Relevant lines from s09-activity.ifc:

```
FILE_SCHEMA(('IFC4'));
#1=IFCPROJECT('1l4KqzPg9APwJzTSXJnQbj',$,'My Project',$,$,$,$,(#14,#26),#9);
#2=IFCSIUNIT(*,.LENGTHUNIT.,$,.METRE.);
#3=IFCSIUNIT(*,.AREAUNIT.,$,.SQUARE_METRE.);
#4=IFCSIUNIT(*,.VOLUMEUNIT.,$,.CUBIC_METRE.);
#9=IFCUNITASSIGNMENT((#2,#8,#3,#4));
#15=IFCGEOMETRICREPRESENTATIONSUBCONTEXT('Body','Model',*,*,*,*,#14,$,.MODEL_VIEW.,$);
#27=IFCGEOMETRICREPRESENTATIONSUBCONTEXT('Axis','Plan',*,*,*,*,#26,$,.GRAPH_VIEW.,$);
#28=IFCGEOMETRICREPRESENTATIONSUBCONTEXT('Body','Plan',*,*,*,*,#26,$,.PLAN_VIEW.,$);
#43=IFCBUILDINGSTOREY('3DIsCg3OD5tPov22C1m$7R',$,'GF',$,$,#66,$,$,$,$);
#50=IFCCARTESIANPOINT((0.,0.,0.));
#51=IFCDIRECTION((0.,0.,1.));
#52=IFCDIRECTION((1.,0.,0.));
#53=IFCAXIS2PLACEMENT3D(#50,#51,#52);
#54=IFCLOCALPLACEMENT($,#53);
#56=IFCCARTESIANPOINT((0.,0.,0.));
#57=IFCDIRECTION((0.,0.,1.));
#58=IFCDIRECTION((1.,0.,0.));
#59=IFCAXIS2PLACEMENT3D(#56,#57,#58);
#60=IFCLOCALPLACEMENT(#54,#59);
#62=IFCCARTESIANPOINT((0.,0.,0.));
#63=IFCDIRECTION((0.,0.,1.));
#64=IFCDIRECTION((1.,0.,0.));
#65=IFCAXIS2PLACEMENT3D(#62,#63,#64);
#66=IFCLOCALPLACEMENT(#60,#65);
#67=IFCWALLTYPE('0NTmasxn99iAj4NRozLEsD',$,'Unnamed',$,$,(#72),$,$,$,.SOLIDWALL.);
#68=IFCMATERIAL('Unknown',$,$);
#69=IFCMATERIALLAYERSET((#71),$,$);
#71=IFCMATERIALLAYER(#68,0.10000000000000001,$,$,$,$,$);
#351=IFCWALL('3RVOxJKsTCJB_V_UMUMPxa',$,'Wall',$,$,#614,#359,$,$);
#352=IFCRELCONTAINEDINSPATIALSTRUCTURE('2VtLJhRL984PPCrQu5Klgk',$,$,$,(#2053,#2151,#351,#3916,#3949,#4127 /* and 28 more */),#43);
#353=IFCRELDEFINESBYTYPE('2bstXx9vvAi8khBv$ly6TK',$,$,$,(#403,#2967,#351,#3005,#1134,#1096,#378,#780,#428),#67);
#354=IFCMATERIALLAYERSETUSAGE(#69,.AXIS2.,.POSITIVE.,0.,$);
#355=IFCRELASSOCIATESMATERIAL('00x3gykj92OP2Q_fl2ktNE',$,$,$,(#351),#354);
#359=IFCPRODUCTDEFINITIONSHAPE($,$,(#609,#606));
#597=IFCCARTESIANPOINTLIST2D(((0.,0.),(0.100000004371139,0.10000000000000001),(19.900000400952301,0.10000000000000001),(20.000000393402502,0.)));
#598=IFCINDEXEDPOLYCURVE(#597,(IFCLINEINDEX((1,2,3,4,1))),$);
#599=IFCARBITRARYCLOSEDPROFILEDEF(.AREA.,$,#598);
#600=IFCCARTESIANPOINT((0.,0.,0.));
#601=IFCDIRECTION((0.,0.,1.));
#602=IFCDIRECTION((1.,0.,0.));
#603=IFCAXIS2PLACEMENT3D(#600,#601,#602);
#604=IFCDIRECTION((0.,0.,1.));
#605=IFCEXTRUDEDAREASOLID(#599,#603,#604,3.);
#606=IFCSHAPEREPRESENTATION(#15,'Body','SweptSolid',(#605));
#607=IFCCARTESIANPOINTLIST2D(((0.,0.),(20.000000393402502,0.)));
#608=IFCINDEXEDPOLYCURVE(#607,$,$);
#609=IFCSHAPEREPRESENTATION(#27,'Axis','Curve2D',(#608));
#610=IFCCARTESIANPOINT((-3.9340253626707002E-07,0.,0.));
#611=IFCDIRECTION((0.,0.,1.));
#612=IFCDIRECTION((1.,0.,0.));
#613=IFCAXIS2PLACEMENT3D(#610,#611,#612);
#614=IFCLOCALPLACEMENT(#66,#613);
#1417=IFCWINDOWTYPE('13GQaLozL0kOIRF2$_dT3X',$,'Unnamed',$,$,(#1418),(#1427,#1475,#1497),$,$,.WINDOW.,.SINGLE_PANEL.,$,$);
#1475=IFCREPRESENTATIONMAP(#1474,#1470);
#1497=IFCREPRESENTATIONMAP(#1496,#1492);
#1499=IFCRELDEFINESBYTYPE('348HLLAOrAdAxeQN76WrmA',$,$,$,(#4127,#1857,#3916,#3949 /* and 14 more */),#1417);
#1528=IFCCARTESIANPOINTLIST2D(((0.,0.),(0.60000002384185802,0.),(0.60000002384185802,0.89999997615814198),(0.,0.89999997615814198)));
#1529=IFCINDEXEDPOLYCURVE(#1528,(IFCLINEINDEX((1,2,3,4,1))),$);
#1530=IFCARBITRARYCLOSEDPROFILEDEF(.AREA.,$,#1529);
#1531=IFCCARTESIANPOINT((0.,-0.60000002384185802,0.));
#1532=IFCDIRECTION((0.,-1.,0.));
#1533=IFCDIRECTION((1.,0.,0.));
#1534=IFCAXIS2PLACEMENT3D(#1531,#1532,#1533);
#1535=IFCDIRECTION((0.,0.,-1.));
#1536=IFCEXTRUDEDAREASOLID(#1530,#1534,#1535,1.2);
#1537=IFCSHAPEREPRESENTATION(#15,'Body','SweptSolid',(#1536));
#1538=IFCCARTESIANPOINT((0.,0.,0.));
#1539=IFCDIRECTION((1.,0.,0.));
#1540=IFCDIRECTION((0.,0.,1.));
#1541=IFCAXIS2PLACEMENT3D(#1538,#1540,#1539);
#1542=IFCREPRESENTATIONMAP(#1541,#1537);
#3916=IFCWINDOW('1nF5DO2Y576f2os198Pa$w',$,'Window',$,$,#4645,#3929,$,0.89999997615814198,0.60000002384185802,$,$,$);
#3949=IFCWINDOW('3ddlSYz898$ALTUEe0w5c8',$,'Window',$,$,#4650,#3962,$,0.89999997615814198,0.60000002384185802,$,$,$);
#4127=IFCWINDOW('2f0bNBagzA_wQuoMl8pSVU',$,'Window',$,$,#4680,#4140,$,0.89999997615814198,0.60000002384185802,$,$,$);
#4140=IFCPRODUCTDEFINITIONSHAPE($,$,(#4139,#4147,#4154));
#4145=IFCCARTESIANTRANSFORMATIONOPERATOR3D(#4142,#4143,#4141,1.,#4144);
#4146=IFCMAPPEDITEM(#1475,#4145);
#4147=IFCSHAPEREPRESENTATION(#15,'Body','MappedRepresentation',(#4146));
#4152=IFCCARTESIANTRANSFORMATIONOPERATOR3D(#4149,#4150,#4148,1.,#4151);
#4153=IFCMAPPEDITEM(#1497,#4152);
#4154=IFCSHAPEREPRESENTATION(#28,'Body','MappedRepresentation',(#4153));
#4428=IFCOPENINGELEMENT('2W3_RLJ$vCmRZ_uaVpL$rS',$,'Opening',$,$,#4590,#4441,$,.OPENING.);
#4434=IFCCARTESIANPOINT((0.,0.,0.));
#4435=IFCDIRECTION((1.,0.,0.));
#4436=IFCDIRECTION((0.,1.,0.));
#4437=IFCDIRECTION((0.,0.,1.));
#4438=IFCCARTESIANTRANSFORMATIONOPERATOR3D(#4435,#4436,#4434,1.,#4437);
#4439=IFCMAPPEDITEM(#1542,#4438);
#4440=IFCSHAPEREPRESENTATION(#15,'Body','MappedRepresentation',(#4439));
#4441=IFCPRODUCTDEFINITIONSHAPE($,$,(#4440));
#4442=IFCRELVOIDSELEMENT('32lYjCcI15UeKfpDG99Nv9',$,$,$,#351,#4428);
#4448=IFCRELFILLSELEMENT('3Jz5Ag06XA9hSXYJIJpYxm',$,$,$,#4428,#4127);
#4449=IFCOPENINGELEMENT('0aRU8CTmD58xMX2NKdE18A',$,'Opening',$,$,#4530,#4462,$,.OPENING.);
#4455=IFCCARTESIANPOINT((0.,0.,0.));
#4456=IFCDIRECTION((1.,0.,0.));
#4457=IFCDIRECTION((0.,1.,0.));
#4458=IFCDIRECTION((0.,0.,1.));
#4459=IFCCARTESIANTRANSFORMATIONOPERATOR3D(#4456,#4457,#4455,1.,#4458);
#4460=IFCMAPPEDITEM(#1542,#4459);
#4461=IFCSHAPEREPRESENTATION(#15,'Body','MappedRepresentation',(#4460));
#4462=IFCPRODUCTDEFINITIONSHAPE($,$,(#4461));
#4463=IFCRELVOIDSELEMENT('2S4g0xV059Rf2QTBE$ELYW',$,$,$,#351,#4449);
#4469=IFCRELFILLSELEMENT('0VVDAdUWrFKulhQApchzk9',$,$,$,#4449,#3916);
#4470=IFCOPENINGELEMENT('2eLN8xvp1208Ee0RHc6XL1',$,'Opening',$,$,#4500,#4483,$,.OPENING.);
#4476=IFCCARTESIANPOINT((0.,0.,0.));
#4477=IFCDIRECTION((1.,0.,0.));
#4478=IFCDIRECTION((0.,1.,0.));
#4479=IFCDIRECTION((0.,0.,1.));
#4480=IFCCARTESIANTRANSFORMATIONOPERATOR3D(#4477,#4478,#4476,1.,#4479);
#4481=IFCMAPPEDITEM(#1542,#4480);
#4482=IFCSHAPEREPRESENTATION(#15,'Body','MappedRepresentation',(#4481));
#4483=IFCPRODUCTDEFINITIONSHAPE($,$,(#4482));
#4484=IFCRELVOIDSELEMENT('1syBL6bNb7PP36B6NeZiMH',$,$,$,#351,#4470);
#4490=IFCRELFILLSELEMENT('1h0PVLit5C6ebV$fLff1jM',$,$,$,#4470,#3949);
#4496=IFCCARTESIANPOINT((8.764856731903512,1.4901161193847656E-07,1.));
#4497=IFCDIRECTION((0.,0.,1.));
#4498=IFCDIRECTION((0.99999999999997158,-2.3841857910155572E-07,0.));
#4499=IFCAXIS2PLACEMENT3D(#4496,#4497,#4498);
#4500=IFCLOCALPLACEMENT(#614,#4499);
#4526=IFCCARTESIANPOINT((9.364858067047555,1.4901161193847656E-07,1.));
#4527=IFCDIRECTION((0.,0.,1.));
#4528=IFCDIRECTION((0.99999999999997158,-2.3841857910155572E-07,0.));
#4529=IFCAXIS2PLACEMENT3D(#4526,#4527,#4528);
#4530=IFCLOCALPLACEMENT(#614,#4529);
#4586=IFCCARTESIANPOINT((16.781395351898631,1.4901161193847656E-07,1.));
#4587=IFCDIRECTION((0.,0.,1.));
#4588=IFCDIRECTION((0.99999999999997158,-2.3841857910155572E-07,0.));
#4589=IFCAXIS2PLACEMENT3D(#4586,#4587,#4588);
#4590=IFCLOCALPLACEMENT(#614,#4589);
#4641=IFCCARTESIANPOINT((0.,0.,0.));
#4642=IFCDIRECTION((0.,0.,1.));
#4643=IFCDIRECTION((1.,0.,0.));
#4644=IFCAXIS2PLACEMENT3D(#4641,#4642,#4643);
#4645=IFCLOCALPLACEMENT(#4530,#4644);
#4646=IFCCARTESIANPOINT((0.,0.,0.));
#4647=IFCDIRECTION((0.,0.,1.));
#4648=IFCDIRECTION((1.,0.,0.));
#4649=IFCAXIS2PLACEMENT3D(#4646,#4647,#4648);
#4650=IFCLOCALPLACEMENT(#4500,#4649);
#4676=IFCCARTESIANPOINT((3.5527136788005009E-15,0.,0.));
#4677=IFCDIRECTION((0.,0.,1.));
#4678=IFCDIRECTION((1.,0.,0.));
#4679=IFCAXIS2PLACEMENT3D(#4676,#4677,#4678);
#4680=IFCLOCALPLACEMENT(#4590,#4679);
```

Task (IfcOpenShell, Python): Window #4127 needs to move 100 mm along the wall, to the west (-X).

```python
import ifcopenshell
import ifcopenshell.api.geometry
import ifcopenshell.util.placement

model = ifcopenshell.open("s09-activity.ifc")

window = model.by_guid("2f0bNBagzA_wQuoMl8pSVU")
opening = window.FillsVoids[0].RelatingOpeningElement
wall = opening.VoidsElements[0].RelatingBuildingElement

wall_matrix = ifcopenshell.util.placement.get_local_placement(wall.ObjectPlacement)
shift = wall_matrix[:3, 0] * -0.1
before = ifcopenshell.util.placement.get_local_placement(window.ObjectPlacement)[:3, 3].copy()

# The window is placed relative to its opening, so it follows when the opening moves.
matrix = ifcopenshell.util.placement.get_local_placement(opening.ObjectPlacement)
matrix[:3, 3] += shift
ifcopenshell.api.geometry.edit_object_placement(
    model, product=opening, matrix=matrix, is_si=False, should_transform_children=True
)

after = ifcopenshell.util.placement.get_local_placement(window.ObjectPlacement)[:3, 3]
print("window moved by", (after - before).round(3) + 0.0)

model.write("s09-activity_v2.ifc")
```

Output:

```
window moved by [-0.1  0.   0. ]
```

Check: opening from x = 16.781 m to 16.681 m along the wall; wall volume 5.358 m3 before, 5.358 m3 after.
